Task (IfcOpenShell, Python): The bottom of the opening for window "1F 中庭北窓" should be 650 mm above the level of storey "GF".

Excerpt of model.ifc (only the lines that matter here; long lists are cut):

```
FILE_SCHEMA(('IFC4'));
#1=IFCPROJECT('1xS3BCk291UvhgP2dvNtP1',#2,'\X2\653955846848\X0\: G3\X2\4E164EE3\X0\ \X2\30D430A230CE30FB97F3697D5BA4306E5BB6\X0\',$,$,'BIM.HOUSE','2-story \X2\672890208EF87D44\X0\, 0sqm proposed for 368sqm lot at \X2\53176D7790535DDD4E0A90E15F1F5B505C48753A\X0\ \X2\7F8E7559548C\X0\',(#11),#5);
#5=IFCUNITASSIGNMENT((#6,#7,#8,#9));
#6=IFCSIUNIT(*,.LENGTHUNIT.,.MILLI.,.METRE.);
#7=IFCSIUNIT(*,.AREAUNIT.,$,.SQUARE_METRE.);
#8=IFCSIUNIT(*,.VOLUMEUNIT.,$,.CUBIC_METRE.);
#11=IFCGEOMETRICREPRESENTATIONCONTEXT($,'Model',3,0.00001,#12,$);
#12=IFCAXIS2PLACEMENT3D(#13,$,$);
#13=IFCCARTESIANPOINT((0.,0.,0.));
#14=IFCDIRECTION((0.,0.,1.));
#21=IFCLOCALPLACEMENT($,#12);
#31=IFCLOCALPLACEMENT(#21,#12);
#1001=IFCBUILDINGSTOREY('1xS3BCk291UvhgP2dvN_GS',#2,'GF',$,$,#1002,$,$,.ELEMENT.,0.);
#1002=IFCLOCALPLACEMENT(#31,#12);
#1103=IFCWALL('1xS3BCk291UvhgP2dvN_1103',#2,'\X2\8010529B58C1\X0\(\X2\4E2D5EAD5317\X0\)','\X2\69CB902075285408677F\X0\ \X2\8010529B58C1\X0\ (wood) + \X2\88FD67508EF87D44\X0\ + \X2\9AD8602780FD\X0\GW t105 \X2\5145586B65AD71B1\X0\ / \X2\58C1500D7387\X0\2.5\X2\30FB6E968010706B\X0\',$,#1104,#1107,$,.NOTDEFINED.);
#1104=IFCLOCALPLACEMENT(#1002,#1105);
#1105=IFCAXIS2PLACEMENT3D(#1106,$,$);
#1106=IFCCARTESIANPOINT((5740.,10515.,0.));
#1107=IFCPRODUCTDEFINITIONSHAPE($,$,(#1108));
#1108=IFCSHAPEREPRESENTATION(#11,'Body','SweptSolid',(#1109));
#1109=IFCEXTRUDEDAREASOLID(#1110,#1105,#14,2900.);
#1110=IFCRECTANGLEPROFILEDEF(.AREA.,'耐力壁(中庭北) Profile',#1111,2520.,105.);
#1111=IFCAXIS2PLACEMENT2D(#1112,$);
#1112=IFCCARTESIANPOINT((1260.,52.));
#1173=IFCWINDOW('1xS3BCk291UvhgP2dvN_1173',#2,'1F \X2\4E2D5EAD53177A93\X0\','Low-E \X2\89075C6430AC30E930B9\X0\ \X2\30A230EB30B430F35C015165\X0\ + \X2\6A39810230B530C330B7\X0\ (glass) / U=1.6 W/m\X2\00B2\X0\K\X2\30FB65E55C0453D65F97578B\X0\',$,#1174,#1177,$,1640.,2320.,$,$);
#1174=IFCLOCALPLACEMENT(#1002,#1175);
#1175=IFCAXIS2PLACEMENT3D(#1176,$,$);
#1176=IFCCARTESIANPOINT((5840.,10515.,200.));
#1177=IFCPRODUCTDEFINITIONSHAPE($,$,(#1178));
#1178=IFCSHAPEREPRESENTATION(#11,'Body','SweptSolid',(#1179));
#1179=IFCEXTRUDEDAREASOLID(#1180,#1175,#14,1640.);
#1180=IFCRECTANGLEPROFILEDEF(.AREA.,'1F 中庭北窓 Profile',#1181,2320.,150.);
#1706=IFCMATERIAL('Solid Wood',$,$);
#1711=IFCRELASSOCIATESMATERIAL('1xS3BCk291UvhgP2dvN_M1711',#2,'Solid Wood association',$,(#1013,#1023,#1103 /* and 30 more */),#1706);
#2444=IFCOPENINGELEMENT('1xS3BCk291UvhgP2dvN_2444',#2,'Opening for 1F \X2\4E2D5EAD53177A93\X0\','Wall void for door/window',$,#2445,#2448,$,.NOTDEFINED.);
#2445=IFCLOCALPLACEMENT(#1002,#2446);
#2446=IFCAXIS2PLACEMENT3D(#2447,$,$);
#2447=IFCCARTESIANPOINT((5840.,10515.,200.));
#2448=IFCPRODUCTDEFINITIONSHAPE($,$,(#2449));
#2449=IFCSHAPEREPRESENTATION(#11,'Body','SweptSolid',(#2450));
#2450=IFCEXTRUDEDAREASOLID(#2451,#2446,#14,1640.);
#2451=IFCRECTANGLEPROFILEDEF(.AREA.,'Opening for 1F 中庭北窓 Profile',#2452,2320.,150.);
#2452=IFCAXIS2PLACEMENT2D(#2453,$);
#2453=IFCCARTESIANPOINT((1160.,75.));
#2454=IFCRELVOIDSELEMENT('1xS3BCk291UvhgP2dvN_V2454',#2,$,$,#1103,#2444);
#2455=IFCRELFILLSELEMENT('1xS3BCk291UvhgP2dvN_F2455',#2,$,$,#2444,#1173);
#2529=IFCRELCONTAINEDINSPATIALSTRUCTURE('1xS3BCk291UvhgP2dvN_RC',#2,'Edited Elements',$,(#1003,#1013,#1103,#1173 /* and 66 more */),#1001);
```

```python
import numpy as np
import ifcopenshell
import ifcopenshell.api.geometry
import ifcopenshell.geom
import ifcopenshell.util.element
import ifcopenshell.util.placement
import ifcopenshell.util.shape
import ifcopenshell.util.unit

model = ifcopenshell.open("model.ifc")
unit_scale = ifcopenshell.util.unit.calculate_unit_scale(model)

window = model.by_id(1173)
opening = window.FillsVoids[0].RelatingOpeningElement
storey = ifcopenshell.util.element.get_container(window, ifc_class="IfcBuildingStorey")
level = ifcopenshell.util.placement.get_local_placement(storey.ObjectPlacement)[2, 3]

# The opening's origin need not be at the sill, so measure its lowest point.
shape = ifcopenshell.geom.create_shape(ifcopenshell.geom.settings(), opening)
bottom = ifcopenshell.util.shape.get_shape_bottom_elevation(shape, shape.geometry) / unit_scale
dz = level + 650.0 - bottom

shift = np.array([0.0, 0.0, dz])
# The window is not placed relative to its opening, so move both.
for product in (opening, window):
    matrix = ifcopenshell.util.placement.get_local_placement(product.ObjectPlacement)
    matrix[:3, 3] += shift
    ifcopenshell.api.geometry.edit_object_placement(model, product=product, matrix=matrix, is_si=False)

print(f"moved by {dz * unit_scale:+.3f} m")

model.write("model_updated.ifc")
```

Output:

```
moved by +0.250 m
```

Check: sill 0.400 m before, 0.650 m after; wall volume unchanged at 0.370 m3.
